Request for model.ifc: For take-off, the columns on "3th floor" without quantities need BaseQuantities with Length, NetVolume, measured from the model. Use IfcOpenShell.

First a look at what the model holds.

```python
import ifcopenshell
import ifcopenshell.util.element
import ifcopenshell.util.unit

model = ifcopenshell.open("model.ifc")
print(model.schema)
for unit_type in ("LENGTHUNIT", "AREAUNIT", "VOLUMEUNIT"):
    print(unit_type, ifcopenshell.util.unit.calculate_unit_scale(model, unit_type))
storey = next(s for s in model.by_type("IfcBuildingStorey") if s.Name == "3th floor")
columns = [e for e in ifcopenshell.util.element.get_decomposition(storey) if e.is_a("IfcColumn")]
for e in sorted(columns, key=lambda e: e.id()):
    print(e.id(), e.is_a(), e.Name, list(ifcopenshell.util.element.get_psets(e, qtos_only=True)), sep=" | ")
```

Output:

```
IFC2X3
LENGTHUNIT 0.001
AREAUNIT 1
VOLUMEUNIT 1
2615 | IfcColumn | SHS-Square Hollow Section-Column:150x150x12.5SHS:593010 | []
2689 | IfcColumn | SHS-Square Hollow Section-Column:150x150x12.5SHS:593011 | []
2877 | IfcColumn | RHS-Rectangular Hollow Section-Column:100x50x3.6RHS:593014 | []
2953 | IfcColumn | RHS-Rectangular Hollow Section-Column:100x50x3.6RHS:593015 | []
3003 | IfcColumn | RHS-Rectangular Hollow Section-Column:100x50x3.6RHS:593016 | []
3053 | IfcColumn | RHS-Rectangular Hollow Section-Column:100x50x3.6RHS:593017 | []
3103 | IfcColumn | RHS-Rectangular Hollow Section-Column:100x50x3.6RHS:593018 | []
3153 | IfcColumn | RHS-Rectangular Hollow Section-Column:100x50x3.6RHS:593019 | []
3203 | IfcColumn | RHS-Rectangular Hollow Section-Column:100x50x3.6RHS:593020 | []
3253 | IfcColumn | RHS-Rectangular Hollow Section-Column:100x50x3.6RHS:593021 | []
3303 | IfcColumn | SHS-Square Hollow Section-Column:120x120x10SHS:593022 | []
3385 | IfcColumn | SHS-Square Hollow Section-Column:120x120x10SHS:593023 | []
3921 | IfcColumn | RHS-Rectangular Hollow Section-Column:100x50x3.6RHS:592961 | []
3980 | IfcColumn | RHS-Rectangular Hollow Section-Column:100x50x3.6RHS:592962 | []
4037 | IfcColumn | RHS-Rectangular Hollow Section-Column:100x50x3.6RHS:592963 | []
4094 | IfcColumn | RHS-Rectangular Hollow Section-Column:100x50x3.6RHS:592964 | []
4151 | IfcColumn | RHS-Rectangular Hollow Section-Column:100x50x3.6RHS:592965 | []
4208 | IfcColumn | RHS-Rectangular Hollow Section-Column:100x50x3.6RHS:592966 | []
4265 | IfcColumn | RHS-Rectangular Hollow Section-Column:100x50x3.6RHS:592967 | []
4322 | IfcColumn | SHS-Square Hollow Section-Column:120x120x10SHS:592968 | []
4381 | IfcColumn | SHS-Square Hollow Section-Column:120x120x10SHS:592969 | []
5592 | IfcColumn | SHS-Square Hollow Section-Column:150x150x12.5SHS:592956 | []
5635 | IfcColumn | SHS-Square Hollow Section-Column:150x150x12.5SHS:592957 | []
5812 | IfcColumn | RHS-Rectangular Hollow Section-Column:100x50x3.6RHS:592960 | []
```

```python
import ifcopenshell
import ifcopenshell.api.pset
import ifcopenshell.geom
import ifcopenshell.util.element
import ifcopenshell.util.shape
import ifcopenshell.util.unit

model = ifcopenshell.open("model.ifc")
unit_scale = ifcopenshell.util.unit.calculate_unit_scale(model)
volume_scale = ifcopenshell.util.unit.calculate_unit_scale(model, "VOLUMEUNIT")
settings = ifcopenshell.geom.settings()

storey = next(s for s in model.by_type("IfcBuildingStorey") if s.Name == "3th floor")
columns = [e for e in ifcopenshell.util.element.get_decomposition(storey) if e.is_a("IfcColumn")]

for e in sorted(columns, key=lambda e: e.id()):
    if ifcopenshell.util.element.get_psets(e, qtos_only=True, should_inherit=False):
        continue
    # Geometry comes back in metres, in the element's own axes.
    shape = ifcopenshell.geom.create_shape(settings, e)
    values = {
        "Length": ifcopenshell.util.shape.get_z(shape.geometry) / unit_scale,
        "NetVolume": ifcopenshell.util.shape.get_volume(shape.geometry) / volume_scale,
    }
    qto = ifcopenshell.api.pset.add_qto(model, product=e, name="BaseQuantities")
    ifcopenshell.api.pset.edit_qto(model, qto=qto, properties=values)
    print(e.id(), {k: round(v, 3) for k, v in values.items()})

model.write("model_updated.ifc")
```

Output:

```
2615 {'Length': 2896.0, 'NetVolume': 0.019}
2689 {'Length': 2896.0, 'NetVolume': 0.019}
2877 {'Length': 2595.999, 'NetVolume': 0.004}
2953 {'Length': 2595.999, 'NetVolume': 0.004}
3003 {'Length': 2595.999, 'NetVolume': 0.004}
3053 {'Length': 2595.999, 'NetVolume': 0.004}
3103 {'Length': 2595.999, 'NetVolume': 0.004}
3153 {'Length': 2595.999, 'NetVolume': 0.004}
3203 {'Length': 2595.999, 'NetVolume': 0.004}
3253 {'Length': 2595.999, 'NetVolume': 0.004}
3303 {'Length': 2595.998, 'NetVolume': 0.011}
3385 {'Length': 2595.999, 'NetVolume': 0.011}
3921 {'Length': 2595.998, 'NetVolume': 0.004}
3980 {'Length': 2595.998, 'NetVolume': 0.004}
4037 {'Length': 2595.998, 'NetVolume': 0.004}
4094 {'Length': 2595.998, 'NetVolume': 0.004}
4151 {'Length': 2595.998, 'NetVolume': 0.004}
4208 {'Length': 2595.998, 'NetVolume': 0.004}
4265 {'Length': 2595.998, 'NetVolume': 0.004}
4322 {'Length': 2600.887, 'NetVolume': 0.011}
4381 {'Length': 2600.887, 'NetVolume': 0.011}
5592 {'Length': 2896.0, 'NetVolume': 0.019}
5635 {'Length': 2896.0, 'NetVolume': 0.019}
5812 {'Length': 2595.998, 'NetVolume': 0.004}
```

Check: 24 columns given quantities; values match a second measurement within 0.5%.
